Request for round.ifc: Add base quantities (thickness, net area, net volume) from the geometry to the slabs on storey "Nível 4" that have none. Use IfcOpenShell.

First a look at what the model holds.

```python
import ifcopenshell
import ifcopenshell.util.element
import ifcopenshell.util.unit

model = ifcopenshell.open("round.ifc")
print(model.schema)
for unit_type in ("LENGTHUNIT", "AREAUNIT", "VOLUMEUNIT"):
    print(unit_type, ifcopenshell.util.unit.calculate_unit_scale(model, unit_type))
storey = next(s for s in model.by_type("IfcBuildingStorey") if s.Name == "Nível 4")
slabs = [e for e in ifcopenshell.util.element.get_decomposition(storey) if e.is_a("IfcSlab")]
for e in sorted(slabs, key=lambda e: e.id()):
    print(e.id(), e.is_a(), e.Name, list(ifcopenshell.util.element.get_psets(e, qtos_only=True)), sep=" | ")
```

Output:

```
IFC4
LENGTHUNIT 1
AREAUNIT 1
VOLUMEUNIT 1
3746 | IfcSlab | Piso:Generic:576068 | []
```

```python
import ifcopenshell
import ifcopenshell.api.pset
import ifcopenshell.geom
import ifcopenshell.util.element
import ifcopenshell.util.shape
import ifcopenshell.util.unit

model = ifcopenshell.open("round.ifc")
unit_scale = ifcopenshell.util.unit.calculate_unit_scale(model)
area_scale = ifcopenshell.util.unit.calculate_unit_scale(model, "AREAUNIT")
volume_scale = ifcopenshell.util.unit.calculate_unit_scale(model, "VOLUMEUNIT")
settings = ifcopenshell.geom.settings()

storey = next(s for s in model.by_type("IfcBuildingStorey") if s.Name == "Nível 4")
slabs = [e for e in ifcopenshell.util.element.get_decomposition(storey) if e.is_a("IfcSlab")]

for e in sorted(slabs, key=lambda e: e.id()):
    if ifcopenshell.util.element.get_psets(e, qtos_only=True, should_inherit=False):
        continue
    # Geometry comes back in metres, in the element's own axes.
    shape = ifcopenshell.geom.create_shape(settings, e)
    values = {
        "Width": ifcopenshell.util.shape.get_z(shape.geometry) / unit_scale,
        "NetArea": ifcopenshell.util.shape.get_footprint_area(shape.geometry) / area_scale,
        "NetVolume": ifcopenshell.util.shape.get_volume(shape.geometry) / volume_scale,
    }
    qto = ifcopenshell.api.pset.add_qto(model, product=e, name="Qto_SlabBaseQuantities")
    ifcopenshell.api.pset.edit_qto(model, qto=qto, properties=values)
    print(e.id(), {k: round(v, 3) for k, v in values.items()})

model.write("round_v2.ifc")
```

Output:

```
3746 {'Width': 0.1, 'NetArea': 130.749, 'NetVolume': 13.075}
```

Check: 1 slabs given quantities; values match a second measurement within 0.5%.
